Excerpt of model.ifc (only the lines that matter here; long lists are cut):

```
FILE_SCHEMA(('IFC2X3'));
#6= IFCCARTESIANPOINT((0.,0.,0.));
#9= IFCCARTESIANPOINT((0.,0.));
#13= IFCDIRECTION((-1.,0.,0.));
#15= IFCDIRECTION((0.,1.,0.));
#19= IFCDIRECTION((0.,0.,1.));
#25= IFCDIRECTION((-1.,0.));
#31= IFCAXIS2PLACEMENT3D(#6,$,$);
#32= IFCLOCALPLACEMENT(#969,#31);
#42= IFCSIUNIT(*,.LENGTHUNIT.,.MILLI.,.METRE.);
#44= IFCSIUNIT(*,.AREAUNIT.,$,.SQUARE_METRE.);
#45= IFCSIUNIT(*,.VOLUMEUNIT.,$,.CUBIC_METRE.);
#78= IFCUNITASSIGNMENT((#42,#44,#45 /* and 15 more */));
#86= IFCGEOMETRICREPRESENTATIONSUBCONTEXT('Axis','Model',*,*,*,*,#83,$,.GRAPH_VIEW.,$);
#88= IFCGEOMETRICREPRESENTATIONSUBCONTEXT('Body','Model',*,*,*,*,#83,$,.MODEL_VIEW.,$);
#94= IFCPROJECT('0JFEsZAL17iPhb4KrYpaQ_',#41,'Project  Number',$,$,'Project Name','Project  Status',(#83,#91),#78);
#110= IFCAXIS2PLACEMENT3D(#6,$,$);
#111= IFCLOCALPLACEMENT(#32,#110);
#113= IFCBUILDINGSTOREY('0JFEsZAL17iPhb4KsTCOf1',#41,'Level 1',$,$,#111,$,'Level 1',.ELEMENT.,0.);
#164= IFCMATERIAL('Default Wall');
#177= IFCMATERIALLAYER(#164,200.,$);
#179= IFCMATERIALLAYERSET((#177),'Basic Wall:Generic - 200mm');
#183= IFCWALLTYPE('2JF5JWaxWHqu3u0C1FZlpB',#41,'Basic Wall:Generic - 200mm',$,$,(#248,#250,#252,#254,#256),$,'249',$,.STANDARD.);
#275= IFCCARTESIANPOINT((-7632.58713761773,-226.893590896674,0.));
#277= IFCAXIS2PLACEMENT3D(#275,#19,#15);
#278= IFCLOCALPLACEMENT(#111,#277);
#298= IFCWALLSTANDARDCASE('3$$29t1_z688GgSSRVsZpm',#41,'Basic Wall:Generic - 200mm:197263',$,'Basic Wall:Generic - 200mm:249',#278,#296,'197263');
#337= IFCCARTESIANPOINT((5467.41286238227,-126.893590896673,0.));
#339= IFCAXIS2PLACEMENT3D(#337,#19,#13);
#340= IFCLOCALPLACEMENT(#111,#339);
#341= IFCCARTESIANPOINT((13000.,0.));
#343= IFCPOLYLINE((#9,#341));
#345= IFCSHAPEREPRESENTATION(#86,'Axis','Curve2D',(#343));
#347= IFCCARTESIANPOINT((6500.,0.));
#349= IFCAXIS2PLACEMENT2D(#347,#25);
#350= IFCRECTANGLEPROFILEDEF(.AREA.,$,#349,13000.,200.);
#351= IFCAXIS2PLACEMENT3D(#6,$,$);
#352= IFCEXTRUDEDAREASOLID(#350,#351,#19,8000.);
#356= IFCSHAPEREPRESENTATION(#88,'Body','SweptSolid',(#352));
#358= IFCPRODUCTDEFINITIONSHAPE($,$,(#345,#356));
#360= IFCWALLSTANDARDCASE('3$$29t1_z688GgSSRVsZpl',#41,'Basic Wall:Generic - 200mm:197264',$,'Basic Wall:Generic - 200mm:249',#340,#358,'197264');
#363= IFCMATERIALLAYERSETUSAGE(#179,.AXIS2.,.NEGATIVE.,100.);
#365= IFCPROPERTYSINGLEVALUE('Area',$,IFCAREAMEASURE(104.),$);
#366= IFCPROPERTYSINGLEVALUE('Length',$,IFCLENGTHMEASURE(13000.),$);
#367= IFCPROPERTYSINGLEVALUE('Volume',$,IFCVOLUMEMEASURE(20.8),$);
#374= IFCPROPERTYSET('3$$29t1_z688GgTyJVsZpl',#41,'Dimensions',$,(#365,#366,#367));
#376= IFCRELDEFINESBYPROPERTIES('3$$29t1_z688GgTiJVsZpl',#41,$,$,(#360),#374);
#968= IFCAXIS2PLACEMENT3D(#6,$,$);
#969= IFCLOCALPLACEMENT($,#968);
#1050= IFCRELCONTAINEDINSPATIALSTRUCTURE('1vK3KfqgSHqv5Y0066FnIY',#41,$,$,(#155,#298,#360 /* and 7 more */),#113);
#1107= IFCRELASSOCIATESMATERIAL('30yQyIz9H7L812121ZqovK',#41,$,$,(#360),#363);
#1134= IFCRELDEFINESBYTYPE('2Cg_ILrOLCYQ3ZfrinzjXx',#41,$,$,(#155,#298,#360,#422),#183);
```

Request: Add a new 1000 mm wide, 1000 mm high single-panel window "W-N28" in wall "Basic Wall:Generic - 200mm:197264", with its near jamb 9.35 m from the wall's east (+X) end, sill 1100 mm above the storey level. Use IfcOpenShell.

```python
import numpy as np
import ifcopenshell
import ifcopenshell.api.feature
import ifcopenshell.api.geometry
import ifcopenshell.api.pset
import ifcopenshell.api.root
import ifcopenshell.api.spatial
import ifcopenshell.api.type
import ifcopenshell.geom
import ifcopenshell.util.element
import ifcopenshell.util.placement
import ifcopenshell.util.representation
import ifcopenshell.util.shape
import ifcopenshell.util.unit

model = ifcopenshell.open("model.ifc")
unit_scale = ifcopenshell.util.unit.calculate_unit_scale(model)
area_scale = ifcopenshell.util.unit.calculate_unit_scale(model, "AREAUNIT")
volume_scale = ifcopenshell.util.unit.calculate_unit_scale(model, "VOLUMEUNIT")
settings = ifcopenshell.geom.settings()


def volume(element):
    """Net volume in cubic metres, openings subtracted."""
    shape = ifcopenshell.geom.create_shape(settings, element)
    return ifcopenshell.util.shape.get_volume(shape.geometry)


wall = model.by_guid("3$$29t1_z688GgSSRVsZpl")
storey = ifcopenshell.util.element.get_container(wall, ifc_class="IfcBuildingStorey")
context = ifcopenshell.util.representation.get_context(model, "Model", "Body", "MODEL_VIEW")
before = volume(wall)

width, height, from_end, sill = 1, 1, 9.35, 1.1  # metres

# The wall runs along its own X axis, and the end named is its -X end.
wall_shape = ifcopenshell.geom.create_shape(settings, wall)
x, y, z = ifcopenshell.util.shape.get_vertices(wall_shape.geometry).T
start = x.min() + from_end
face, thickness = float(y.min()), float(y.max() - y.min())
wall_matrix = ifcopenshell.util.placement.get_local_placement(wall.ObjectPlacement)
level = ifcopenshell.util.placement.get_local_placement(storey.ObjectPlacement)[2, 3]


def in_wall(x, y):
    """Placement at x, y metres in the wall's axes, at sill height."""
    matrix = wall_matrix.copy()
    matrix[:, 3] = wall_matrix @ np.array([x / unit_scale, y / unit_scale, 0.0, 1.0])
    matrix[2, 3] = level + sill / unit_scale
    return matrix


# Opening: a box that overshoots both wall faces by 50 mm.
opening = ifcopenshell.api.root.create_entity(model, ifc_class="IfcOpeningElement")
box = ifcopenshell.api.geometry.add_wall_representation(
    model, context=context, length=width, height=height, thickness=thickness + 0.1
)
ifcopenshell.api.geometry.assign_representation(model, product=opening, representation=box)
ifcopenshell.api.geometry.edit_object_placement(model, product=opening, matrix=in_wall(start, face - 0.05), is_si=False)
ifcopenshell.api.feature.add_feature(model, feature=opening, element=wall)

window = ifcopenshell.api.root.create_entity(model, ifc_class="IfcWindow", name="W-N28")
window.OverallWidth, window.OverallHeight = width / unit_scale, height / unit_scale
body = ifcopenshell.api.geometry.add_window_representation(
    model,
    context=context,
    overall_width=window.OverallWidth,
    overall_height=window.OverallHeight,
    partition_type="SINGLE_PANEL",
)
ifcopenshell.api.geometry.assign_representation(model, product=window, representation=body)
ifcopenshell.api.spatial.assign_container(model, products=[window], relating_structure=storey)
fills = ifcopenshell.api.feature.add_filling(model, opening=opening, element=window)
fills.OwnerHistory = window.OwnerHistory  # required in IFC2X3

# IFC2X3 keeps the operation on the window style.
style = ifcopenshell.api.root.create_entity(model, ifc_class="IfcWindowStyle", name="W-N28")
style.OperationType, style.ConstructionType = "SINGLE_PANEL", "NOTDEFINED"
style.ParameterTakesPrecedence = style.Sizeable = False
ifcopenshell.api.type.assign_type(model, related_objects=[window], relating_type=style)

# Centre the window in the wall's thickness.
ifcopenshell.api.geometry.edit_object_placement(model, product=window, matrix=in_wall(start, face), is_si=False)
window_shape = ifcopenshell.geom.create_shape(settings, window)
depth = ifcopenshell.util.shape.get_vertices(window_shape.geometry)[:, 1]
offset = face + thickness / 2 - (depth.min() + depth.max()) / 2
ifcopenshell.api.geometry.edit_object_placement(model, product=window, matrix=in_wall(start, offset), is_si=False)

after = volume(wall)

# Update the wall's stored quantities.
pset = model.by_id(ifcopenshell.util.element.get_pset(wall, "Dimensions", should_inherit=False)["id"])
ifcopenshell.api.pset.edit_pset(model, pset=pset, properties={
    "Area": model.create_entity("IfcAreaMeasure", after / thickness / area_scale),
    "Volume": model.create_entity("IfcVolumeMeasure", after / volume_scale),
})

print(f"wall volume {before:.3f} -> {after:.3f} m3")

model.write("model_rev.ifc")
```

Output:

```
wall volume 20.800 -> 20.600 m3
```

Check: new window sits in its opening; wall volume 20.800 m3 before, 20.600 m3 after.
